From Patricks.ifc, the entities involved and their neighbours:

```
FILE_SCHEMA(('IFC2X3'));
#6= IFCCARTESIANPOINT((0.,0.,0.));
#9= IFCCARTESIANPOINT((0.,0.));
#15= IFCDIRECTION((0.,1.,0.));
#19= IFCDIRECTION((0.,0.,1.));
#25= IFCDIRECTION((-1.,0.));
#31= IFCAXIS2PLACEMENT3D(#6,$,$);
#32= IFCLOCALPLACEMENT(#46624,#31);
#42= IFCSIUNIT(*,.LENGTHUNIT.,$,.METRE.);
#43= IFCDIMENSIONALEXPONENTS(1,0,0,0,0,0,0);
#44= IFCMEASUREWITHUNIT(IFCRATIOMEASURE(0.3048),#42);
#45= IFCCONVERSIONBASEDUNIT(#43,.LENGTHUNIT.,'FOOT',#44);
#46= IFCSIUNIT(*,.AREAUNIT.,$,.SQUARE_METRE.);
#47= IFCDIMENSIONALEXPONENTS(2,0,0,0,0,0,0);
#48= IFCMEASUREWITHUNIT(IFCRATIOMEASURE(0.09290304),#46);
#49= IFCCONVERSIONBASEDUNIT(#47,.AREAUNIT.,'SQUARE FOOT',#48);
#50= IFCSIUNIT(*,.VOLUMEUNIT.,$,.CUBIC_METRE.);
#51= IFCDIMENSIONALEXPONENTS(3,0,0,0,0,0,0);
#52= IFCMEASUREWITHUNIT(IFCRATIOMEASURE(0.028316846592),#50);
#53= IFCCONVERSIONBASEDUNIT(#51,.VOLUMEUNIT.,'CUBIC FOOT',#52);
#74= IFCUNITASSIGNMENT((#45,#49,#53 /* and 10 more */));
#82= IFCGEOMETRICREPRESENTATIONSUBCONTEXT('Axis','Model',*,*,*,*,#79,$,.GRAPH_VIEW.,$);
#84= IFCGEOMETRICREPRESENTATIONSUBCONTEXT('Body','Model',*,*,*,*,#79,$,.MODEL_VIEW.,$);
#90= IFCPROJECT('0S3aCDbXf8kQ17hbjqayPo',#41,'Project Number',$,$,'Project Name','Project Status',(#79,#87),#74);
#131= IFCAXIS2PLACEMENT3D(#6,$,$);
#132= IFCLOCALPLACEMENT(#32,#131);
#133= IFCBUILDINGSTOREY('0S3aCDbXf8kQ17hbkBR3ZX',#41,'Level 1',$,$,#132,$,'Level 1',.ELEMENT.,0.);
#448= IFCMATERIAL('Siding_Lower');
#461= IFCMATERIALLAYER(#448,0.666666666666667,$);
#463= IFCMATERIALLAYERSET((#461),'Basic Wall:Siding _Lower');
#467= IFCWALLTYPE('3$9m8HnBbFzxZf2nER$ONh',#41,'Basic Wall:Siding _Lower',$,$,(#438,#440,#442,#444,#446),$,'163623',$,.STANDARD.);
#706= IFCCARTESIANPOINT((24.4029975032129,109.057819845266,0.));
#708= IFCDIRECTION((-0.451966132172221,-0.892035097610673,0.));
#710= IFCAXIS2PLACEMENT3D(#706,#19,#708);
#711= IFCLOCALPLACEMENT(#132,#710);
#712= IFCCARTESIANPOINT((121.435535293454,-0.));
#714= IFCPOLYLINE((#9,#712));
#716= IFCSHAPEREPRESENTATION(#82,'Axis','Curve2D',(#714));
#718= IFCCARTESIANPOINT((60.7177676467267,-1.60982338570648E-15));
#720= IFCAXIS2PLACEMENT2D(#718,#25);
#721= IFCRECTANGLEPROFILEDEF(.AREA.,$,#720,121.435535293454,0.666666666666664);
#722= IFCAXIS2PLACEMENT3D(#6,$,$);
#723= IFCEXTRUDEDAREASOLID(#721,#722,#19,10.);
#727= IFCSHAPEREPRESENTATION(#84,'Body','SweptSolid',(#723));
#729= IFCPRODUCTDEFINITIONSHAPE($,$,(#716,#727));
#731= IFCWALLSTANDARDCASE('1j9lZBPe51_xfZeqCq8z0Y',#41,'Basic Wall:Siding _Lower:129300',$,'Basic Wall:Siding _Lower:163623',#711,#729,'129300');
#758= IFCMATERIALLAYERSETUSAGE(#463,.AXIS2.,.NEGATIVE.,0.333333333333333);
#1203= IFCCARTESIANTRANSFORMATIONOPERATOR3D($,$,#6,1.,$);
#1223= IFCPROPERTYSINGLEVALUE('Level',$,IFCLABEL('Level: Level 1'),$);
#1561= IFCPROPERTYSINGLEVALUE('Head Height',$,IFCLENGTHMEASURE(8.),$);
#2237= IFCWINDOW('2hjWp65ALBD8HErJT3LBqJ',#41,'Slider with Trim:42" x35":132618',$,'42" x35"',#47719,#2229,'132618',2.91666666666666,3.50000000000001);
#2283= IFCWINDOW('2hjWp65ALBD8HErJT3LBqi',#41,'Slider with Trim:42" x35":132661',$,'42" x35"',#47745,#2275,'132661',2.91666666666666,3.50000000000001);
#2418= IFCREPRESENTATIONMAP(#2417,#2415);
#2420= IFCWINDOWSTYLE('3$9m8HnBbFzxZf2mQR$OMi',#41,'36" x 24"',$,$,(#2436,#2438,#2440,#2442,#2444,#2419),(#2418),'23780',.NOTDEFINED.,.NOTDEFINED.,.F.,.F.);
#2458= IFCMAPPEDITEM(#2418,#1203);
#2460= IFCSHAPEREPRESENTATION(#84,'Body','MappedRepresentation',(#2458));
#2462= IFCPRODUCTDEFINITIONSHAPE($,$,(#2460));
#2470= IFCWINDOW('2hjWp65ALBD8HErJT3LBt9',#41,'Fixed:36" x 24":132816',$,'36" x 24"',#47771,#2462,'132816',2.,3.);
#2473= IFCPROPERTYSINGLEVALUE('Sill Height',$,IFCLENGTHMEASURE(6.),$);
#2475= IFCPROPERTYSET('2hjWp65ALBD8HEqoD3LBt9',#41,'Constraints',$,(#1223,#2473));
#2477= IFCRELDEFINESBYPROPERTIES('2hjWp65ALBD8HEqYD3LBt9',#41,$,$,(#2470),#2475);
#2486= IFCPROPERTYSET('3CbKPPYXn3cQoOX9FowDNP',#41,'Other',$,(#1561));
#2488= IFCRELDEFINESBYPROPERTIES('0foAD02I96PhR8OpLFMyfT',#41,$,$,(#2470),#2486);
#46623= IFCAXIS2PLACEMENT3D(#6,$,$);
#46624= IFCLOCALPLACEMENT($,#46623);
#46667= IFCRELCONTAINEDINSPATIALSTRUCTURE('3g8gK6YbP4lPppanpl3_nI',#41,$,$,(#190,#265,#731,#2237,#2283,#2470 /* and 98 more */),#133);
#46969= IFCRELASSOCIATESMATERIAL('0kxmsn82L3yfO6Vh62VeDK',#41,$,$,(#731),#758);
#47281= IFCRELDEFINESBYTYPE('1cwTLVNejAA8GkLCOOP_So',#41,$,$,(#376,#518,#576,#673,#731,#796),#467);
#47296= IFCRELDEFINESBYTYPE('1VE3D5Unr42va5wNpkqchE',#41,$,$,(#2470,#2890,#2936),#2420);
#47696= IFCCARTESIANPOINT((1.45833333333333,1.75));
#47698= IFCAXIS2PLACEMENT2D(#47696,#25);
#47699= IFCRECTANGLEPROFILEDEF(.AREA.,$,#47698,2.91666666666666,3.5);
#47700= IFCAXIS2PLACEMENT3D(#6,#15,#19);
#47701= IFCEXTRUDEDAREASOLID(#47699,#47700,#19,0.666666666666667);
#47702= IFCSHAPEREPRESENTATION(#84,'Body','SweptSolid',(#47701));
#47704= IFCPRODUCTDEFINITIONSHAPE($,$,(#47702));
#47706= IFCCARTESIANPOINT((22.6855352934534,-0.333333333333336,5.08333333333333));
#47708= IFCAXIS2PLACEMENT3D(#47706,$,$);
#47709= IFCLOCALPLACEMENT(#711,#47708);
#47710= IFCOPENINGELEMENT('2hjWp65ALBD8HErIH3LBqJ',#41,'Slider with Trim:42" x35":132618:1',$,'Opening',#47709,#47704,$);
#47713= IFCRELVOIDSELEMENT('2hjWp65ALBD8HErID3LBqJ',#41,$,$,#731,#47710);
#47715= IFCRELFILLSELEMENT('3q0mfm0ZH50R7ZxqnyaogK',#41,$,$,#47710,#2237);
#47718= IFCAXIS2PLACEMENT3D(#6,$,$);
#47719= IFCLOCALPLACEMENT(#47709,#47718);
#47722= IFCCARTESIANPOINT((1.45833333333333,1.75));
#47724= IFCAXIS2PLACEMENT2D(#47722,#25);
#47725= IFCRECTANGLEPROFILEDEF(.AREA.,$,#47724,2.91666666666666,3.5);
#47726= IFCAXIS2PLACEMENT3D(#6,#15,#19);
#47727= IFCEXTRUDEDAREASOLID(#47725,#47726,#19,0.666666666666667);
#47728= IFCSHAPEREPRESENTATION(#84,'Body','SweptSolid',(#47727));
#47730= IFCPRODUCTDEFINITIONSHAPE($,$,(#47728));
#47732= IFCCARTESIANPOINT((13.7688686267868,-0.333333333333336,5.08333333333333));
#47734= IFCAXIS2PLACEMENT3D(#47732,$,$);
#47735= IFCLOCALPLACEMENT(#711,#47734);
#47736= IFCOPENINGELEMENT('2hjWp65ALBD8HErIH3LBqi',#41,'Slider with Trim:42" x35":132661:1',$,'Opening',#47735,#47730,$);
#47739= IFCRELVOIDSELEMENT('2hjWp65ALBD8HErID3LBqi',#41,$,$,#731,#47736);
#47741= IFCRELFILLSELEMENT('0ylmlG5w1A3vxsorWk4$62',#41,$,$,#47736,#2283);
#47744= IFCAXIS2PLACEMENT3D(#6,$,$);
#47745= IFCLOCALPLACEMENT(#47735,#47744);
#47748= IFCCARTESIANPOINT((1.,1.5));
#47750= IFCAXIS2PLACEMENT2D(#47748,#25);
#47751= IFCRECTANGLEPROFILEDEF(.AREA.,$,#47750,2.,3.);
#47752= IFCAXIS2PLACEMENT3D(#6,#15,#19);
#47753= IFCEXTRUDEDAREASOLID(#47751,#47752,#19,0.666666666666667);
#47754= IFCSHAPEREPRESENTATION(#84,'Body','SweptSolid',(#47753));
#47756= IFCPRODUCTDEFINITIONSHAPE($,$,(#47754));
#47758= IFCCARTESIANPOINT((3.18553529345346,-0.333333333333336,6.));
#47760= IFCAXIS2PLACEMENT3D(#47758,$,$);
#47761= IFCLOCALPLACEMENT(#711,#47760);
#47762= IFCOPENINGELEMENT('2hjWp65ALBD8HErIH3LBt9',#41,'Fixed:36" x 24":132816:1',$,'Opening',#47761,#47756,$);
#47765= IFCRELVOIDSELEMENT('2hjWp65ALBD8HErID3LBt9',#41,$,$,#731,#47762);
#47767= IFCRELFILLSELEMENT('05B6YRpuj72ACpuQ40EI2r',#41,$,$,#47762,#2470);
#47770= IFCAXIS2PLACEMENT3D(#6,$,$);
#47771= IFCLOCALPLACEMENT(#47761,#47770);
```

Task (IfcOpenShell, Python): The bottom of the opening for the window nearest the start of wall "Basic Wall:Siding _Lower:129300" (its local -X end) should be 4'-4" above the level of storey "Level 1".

```python
import numpy as np
import ifcopenshell
import ifcopenshell.api.geometry
import ifcopenshell.api.pset
import ifcopenshell.geom
import ifcopenshell.util.element
import ifcopenshell.util.placement
import ifcopenshell.util.shape
import ifcopenshell.util.unit

model = ifcopenshell.open("Patricks.ifc")
unit_scale = ifcopenshell.util.unit.calculate_unit_scale(model)

window = model.by_guid("2hjWp65ALBD8HErJT3LBt9")
opening = window.FillsVoids[0].RelatingOpeningElement
storey = ifcopenshell.util.element.get_container(window, ifc_class="IfcBuildingStorey")
level = ifcopenshell.util.placement.get_local_placement(storey.ObjectPlacement)[2, 3]

# The opening's origin need not be at the sill, so measure its lowest point.
shape = ifcopenshell.geom.create_shape(ifcopenshell.geom.settings(), opening)
bottom = ifcopenshell.util.shape.get_shape_bottom_elevation(shape, shape.geometry) / unit_scale
dz = level + 52 * 0.0254 / unit_scale - bottom

shift = np.array([0.0, 0.0, dz])
# The window is placed relative to its opening, so it follows when the opening moves.
matrix = ifcopenshell.util.placement.get_local_placement(opening.ObjectPlacement)
matrix[:3, 3] += shift
ifcopenshell.api.geometry.edit_object_placement(
    model, product=opening, matrix=matrix, is_si=False, should_transform_children=True
)

# Keep the stored heights in step.
pset = model.by_id(ifcopenshell.util.element.get_pset(window, "Constraints", should_inherit=False)["id"])
ifcopenshell.api.pset.edit_pset(model, pset=pset, properties={
    "Sill Height": model.create_entity("IfcLengthMeasure", ifcopenshell.util.element.get_pset(window, "Constraints", "Sill Height") + dz),
})
pset = model.by_id(ifcopenshell.util.element.get_pset(window, "Other", should_inherit=False)["id"])
ifcopenshell.api.pset.edit_pset(model, pset=pset, properties={
    "Head Height": model.create_entity("IfcLengthMeasure", ifcopenshell.util.element.get_pset(window, "Other", "Head Height") + dz),
})

print(f"moved by {dz * unit_scale:+.3f} m")

model.write("Patricks_v2.ifc")
```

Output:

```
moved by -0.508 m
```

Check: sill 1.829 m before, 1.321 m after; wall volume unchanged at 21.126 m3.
